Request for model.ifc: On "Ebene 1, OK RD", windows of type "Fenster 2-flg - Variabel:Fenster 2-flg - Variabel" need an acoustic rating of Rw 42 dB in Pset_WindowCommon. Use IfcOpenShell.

First a look at what the model holds.

```python
import ifcopenshell
import ifcopenshell.util.element

model = ifcopenshell.open("model.ifc")
print(model.schema)
storey = next(s for s in model.by_type("IfcBuildingStorey") if s.Name == "Ebene 1, OK RD")
windows = [e for e in ifcopenshell.util.element.get_decomposition(storey) if e.is_a("IfcWindow")]
seen = {}
for e in windows:
    element_type = ifcopenshell.util.element.get_type(e)
    key = (element_type.Name if element_type != e and element_type else None, ifcopenshell.util.element.get_pset(e, "Pset_WindowCommon", "AcousticRating"))
    seen[key] = seen.get(key, 0) + 1
for (name, value), count in sorted(seen.items(), key=str):
    print(count, "x", name, "|", value)
```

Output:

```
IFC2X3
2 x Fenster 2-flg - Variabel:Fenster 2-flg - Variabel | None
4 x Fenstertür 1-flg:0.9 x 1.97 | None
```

```python
import ifcopenshell
import ifcopenshell.api.pset
import ifcopenshell.util.element

model = ifcopenshell.open("model.ifc")

storey = next(s for s in model.by_type("IfcBuildingStorey") if s.Name == "Ebene 1, OK RD")
windows = [e for e in ifcopenshell.util.element.get_decomposition(storey) if e.is_a("IfcWindow")]

count = 0
for e in windows:
    element_type = ifcopenshell.util.element.get_type(e)
    if element_type in (None, e) or element_type.Name != "Fenster 2-flg - Variabel:Fenster 2-flg - Variabel":
        continue
    # add_pset returns the element's existing set when there is one.
    pset = ifcopenshell.api.pset.add_pset(model, product=e, name="Pset_WindowCommon")
    ifcopenshell.api.pset.edit_pset(model, pset=pset, properties={"AcousticRating": "Rw 42 dB"})
    count += 1

print(count, "windows updated")

model.write("model-out.ifc")
```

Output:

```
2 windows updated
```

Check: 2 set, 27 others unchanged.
